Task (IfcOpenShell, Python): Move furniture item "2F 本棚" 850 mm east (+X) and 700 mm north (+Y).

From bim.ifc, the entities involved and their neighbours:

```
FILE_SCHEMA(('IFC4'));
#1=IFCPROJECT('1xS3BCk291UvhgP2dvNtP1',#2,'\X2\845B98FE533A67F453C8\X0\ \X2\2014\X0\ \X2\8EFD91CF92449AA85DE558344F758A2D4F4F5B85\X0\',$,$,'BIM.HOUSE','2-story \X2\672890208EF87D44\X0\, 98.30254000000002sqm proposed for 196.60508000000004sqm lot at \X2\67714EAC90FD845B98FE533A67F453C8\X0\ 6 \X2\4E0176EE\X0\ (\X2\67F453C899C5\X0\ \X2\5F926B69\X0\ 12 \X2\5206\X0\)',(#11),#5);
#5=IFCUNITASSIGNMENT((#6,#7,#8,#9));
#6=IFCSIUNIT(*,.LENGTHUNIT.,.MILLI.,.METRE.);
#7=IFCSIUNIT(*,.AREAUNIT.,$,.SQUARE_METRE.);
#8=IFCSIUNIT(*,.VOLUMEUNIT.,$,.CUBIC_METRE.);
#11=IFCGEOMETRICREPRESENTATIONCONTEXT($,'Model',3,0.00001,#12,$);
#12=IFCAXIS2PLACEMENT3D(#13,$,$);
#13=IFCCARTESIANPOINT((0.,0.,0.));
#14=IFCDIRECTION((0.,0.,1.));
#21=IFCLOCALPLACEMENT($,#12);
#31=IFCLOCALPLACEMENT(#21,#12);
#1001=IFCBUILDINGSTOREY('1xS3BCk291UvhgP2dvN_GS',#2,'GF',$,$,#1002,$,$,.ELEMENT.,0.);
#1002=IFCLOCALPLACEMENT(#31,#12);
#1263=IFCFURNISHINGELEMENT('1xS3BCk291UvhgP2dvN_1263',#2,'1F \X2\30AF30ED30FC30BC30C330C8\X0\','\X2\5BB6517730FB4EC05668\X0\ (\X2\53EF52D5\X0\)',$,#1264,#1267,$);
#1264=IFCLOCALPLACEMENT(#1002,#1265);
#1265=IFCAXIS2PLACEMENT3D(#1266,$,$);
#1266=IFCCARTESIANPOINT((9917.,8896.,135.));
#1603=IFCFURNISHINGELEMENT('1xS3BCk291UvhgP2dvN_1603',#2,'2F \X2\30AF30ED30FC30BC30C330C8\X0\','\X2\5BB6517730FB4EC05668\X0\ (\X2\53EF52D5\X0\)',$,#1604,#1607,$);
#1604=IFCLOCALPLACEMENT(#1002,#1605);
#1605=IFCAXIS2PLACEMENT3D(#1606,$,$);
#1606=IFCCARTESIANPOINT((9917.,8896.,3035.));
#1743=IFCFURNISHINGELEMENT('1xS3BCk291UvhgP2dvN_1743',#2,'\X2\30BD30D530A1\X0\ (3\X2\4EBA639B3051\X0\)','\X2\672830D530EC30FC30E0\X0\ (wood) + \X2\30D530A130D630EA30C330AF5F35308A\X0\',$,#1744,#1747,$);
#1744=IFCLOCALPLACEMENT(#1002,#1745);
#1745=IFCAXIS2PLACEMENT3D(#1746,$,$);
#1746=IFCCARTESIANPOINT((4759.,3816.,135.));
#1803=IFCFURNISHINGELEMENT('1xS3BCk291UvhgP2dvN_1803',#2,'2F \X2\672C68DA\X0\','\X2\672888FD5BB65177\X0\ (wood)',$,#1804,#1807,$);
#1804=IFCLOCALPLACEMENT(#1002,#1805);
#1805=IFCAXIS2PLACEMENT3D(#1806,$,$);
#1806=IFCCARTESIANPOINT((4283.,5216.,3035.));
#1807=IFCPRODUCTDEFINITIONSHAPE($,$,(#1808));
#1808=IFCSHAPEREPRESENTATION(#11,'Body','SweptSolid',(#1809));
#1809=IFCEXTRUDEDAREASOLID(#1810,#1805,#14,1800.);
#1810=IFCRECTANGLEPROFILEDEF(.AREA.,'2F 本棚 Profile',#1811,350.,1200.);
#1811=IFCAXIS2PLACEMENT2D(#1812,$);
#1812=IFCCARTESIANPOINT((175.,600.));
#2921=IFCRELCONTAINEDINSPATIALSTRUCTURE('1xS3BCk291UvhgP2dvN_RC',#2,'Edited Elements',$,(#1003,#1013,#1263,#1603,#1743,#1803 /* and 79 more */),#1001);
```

```python
import ifcopenshell
import ifcopenshell.api.geometry
import ifcopenshell.util.placement
import ifcopenshell.util.unit

model = ifcopenshell.open("bim.ifc")
unit_scale = ifcopenshell.util.unit.calculate_unit_scale(model)

item = model.by_guid("1xS3BCk291UvhgP2dvN_1803")
matrix = ifcopenshell.util.placement.get_local_placement(item.ObjectPlacement)
matrix[0, 3] += 0.85 / unit_scale
matrix[1, 3] += 0.7 / unit_scale
ifcopenshell.api.geometry.edit_object_placement(model, product=item, matrix=matrix, is_si=False)

print(ifcopenshell.util.placement.get_local_placement(item.ObjectPlacement).round(3) + 0.0)

model.write("bim_edited.ifc")
```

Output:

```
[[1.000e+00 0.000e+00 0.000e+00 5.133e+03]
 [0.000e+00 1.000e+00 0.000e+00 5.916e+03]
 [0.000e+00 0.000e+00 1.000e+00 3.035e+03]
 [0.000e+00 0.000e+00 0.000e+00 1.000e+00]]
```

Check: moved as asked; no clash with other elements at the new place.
